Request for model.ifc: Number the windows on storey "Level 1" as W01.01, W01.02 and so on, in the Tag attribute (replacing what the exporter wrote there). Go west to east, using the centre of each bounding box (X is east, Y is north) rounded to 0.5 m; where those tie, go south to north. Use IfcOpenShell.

First a look at what the model holds.

```python
import ifcopenshell
import ifcopenshell.util.element
import ifcopenshell.util.placement

model = ifcopenshell.open("model.ifc")
print(model.schema)
storey = next(s for s in model.by_type("IfcBuildingStorey") if s.Name == "Level 1")
windows = [e for e in ifcopenshell.util.element.get_decomposition(storey) if e.is_a("IfcWindow")]
for e in sorted(windows, key=lambda e: e.id()):
    origin = ifcopenshell.util.placement.get_local_placement(e.ObjectPlacement)[:3, 3]
    print(e.id(), e.Tag, e.Name, origin.round(2) + 0.0, sep=" | ")
```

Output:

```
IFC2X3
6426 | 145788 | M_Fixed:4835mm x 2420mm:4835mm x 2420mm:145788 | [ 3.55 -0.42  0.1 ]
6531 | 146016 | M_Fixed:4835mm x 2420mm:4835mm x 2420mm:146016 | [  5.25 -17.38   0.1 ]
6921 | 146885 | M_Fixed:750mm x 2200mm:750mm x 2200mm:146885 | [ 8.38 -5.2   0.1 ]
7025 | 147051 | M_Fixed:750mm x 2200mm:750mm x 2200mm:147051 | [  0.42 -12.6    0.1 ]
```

```python
import ifcopenshell
import ifcopenshell.geom
import ifcopenshell.util.element
import ifcopenshell.util.shape

model = ifcopenshell.open("model.ifc")
settings = ifcopenshell.geom.settings()
settings.set("use-world-coords", True)


def centre(element):
    shape = ifcopenshell.geom.create_shape(settings, element)
    return ifcopenshell.util.shape.get_bbox_centroid(shape.geometry)


storey = next(s for s in model.by_type("IfcBuildingStorey") if s.Name == "Level 1")
windows = [e for e in ifcopenshell.util.element.get_decomposition(storey) if e.is_a("IfcWindow")]

# Insertion points can sit at a corner or the storey origin, so sort by the geometry (in metres).
centres = {e: centre(e) for e in windows}
windows.sort(key=lambda e: (round(centres[e][0] / 0.5), centres[e][1]))

for i, e in enumerate(windows, start=1):
    number = f"W01.{i:02d}"
    e.Tag = number
    print(e.id(), number)

model.write("model_updated.ifc")
```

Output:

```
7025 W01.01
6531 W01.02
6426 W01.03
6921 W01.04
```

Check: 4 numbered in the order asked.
